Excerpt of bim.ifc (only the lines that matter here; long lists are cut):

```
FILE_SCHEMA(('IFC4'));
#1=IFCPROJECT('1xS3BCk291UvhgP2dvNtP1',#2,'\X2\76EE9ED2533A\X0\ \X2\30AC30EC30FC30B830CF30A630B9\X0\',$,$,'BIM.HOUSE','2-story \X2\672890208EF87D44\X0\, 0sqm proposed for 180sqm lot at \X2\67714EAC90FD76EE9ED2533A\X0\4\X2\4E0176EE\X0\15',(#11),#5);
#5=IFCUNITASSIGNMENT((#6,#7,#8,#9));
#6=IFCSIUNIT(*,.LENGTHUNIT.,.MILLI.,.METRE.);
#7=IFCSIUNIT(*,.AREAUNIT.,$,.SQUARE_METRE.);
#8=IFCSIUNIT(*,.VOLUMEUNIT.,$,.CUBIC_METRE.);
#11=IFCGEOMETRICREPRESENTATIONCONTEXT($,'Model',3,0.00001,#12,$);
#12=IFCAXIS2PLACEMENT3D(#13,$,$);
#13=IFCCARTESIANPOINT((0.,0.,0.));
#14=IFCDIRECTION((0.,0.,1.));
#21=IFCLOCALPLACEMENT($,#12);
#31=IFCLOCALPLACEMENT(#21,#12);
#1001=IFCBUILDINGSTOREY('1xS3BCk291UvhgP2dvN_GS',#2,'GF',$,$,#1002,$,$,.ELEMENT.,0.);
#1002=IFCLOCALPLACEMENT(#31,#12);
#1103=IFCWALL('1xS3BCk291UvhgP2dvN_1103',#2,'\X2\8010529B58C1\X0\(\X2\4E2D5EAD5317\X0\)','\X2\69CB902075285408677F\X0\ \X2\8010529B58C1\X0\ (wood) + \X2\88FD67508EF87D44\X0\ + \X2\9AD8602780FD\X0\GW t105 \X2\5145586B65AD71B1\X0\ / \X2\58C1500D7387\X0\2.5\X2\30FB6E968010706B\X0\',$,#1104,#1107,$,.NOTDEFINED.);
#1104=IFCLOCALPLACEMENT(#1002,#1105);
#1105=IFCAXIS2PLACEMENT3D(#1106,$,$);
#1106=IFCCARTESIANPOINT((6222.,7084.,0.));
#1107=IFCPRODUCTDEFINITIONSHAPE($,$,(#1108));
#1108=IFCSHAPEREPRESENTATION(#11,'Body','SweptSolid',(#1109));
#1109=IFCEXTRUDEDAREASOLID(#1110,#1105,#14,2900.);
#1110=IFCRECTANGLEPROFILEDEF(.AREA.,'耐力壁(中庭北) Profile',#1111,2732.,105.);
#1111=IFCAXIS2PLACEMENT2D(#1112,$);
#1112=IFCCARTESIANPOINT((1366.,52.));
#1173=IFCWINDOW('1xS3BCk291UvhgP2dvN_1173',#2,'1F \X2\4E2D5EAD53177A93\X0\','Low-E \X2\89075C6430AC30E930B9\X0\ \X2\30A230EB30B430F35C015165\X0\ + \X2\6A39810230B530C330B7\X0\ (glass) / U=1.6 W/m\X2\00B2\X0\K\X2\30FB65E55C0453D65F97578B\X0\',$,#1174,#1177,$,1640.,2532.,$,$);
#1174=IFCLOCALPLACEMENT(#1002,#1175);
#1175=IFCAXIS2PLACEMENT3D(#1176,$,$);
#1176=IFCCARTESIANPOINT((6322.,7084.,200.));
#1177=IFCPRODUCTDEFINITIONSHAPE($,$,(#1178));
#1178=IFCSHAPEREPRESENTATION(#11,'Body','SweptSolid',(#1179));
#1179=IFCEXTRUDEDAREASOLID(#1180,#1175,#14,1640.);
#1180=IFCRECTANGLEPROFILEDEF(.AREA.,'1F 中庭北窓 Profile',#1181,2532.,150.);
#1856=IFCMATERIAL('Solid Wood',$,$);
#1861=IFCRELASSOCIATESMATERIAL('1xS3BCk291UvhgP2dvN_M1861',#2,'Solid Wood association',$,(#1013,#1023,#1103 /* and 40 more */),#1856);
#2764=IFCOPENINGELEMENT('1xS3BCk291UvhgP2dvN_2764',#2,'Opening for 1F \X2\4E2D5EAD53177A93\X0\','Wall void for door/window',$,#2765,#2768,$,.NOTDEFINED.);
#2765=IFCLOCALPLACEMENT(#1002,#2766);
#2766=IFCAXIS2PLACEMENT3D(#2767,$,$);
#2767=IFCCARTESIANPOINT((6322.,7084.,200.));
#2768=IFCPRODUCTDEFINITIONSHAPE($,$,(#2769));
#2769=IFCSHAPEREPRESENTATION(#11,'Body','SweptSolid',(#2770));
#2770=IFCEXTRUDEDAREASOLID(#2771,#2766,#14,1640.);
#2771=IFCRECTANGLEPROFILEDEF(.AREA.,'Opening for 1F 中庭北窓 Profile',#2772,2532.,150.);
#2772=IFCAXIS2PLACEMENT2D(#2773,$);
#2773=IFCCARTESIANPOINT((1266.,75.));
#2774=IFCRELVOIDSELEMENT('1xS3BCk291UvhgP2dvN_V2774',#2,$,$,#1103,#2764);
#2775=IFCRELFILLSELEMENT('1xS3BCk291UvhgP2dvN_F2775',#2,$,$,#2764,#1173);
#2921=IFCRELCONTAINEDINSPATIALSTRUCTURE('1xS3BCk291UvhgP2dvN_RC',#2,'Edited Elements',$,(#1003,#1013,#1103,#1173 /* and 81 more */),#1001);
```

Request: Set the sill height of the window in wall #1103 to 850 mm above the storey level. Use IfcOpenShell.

```python
import numpy as np
import ifcopenshell
import ifcopenshell.api.geometry
import ifcopenshell.geom
import ifcopenshell.util.element
import ifcopenshell.util.placement
import ifcopenshell.util.shape
import ifcopenshell.util.unit

model = ifcopenshell.open("bim.ifc")
unit_scale = ifcopenshell.util.unit.calculate_unit_scale(model)

window = model.by_id(1173)
opening = window.FillsVoids[0].RelatingOpeningElement
storey = ifcopenshell.util.element.get_container(window, ifc_class="IfcBuildingStorey")
level = ifcopenshell.util.placement.get_local_placement(storey.ObjectPlacement)[2, 3]

# The opening's origin need not be at the sill, so measure its lowest point.
shape = ifcopenshell.geom.create_shape(ifcopenshell.geom.settings(), opening)
bottom = ifcopenshell.util.shape.get_shape_bottom_elevation(shape, shape.geometry) / unit_scale
dz = level + 850.0 - bottom

shift = np.array([0.0, 0.0, dz])
# The window is not placed relative to its opening, so move both.
for product in (opening, window):
    matrix = ifcopenshell.util.placement.get_local_placement(product.ObjectPlacement)
    matrix[:3, 3] += shift
    ifcopenshell.api.geometry.edit_object_placement(model, product=product, matrix=matrix, is_si=False)

print(f"moved by {dz * unit_scale:+.3f} m")

model.write("bim_v2.ifc")
```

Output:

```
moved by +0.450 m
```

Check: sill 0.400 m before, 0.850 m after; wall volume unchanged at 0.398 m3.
